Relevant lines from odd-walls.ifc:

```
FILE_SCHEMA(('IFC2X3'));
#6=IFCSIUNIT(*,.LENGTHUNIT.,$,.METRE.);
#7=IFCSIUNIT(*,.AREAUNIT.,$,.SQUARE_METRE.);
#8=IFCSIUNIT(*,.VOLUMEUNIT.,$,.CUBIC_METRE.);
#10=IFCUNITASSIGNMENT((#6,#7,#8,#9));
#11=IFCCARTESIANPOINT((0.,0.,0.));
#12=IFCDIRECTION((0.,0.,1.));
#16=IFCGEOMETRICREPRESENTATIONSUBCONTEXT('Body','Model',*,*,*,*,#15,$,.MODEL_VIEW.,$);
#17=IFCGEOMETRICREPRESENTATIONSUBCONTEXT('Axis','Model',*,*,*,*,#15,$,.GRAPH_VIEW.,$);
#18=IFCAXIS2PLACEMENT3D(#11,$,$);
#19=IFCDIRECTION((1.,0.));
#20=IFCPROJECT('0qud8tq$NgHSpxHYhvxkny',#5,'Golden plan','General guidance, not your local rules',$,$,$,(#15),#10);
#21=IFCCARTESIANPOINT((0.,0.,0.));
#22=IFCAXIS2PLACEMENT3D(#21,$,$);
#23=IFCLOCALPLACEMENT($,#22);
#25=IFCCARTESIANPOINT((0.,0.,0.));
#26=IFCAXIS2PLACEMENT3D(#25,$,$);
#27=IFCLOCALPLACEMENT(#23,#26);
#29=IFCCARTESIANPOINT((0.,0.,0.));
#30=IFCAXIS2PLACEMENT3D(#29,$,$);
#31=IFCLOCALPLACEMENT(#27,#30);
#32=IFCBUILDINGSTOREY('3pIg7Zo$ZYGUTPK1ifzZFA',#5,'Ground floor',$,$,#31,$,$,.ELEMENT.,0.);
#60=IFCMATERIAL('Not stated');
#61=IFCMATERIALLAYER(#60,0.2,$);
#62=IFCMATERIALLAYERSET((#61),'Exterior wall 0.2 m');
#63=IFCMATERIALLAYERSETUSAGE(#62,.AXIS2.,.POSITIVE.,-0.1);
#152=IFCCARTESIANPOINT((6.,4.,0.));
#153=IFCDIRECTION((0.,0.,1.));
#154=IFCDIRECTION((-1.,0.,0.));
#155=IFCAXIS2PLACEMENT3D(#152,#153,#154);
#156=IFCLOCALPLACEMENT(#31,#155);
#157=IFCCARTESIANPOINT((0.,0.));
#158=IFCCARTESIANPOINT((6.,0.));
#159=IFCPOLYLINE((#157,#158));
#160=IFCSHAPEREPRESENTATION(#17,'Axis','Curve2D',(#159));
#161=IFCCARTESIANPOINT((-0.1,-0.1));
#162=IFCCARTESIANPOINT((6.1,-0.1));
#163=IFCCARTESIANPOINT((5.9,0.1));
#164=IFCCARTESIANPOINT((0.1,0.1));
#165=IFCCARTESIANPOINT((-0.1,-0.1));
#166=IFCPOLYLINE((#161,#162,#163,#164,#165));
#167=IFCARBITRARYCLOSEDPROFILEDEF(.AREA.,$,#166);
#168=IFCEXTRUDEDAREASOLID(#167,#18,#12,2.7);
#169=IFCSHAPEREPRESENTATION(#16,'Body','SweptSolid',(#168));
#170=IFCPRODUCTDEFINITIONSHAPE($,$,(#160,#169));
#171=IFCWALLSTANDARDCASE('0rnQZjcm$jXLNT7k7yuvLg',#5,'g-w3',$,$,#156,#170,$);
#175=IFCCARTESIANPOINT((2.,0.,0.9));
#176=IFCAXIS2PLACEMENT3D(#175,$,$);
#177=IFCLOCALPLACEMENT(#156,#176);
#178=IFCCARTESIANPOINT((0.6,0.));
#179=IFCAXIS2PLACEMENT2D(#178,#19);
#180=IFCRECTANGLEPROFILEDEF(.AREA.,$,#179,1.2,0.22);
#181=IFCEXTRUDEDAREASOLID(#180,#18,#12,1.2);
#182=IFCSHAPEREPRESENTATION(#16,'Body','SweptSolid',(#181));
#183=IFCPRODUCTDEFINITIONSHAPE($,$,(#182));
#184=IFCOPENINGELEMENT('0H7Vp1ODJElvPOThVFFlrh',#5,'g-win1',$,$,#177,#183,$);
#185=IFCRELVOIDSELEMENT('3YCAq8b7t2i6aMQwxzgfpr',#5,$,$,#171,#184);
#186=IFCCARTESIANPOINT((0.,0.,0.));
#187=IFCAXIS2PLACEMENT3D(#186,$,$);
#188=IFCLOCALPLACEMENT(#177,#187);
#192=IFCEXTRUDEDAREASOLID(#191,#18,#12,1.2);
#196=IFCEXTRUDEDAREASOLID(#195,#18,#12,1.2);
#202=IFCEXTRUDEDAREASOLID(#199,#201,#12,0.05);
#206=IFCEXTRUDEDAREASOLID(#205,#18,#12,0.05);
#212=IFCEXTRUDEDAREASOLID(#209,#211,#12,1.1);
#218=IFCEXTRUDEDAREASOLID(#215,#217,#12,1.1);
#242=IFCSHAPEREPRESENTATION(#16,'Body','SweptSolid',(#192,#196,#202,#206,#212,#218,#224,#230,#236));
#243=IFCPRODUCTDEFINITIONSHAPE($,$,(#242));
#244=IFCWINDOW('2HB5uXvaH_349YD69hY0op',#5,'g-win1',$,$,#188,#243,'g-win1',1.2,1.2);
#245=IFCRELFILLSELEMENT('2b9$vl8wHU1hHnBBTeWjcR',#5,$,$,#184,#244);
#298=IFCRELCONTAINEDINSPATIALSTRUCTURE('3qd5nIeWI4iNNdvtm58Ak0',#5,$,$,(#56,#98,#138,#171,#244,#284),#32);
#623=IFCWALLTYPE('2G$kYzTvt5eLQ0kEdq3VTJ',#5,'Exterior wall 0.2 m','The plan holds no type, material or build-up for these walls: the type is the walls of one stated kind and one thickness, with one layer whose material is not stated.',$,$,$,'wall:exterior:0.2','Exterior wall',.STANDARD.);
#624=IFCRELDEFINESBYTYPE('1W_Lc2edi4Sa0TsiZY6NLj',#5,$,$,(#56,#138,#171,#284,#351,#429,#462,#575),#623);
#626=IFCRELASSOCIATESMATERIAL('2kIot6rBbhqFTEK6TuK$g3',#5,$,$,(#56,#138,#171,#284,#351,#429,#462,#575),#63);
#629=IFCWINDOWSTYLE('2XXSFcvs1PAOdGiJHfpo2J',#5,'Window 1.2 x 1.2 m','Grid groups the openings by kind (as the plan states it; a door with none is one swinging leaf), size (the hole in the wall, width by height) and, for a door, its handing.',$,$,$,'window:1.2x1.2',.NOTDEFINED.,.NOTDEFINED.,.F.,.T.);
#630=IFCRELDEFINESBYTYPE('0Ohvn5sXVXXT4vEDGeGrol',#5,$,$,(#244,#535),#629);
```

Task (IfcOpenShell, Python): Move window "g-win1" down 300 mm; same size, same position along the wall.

```python
import numpy as np
import ifcopenshell
import ifcopenshell.api.geometry
import ifcopenshell.util.placement
import ifcopenshell.util.unit

model = ifcopenshell.open("odd-walls.ifc")
unit_scale = ifcopenshell.util.unit.calculate_unit_scale(model)

window = model.by_guid("2HB5uXvaH_349YD69hY0op")
opening = window.FillsVoids[0].RelatingOpeningElement
dz = -0.3 / unit_scale

shift = np.array([0.0, 0.0, dz])
# The window is placed relative to its opening, so it follows when the opening moves.
matrix = ifcopenshell.util.placement.get_local_placement(opening.ObjectPlacement)
matrix[:3, 3] += shift
ifcopenshell.api.geometry.edit_object_placement(
    model, product=opening, matrix=matrix, is_si=False, should_transform_children=True
)

print(f"moved by {dz * unit_scale:+.3f} m")

model.write("odd-walls_rev.ifc")
```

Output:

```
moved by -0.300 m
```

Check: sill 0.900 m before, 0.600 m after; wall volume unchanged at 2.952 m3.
